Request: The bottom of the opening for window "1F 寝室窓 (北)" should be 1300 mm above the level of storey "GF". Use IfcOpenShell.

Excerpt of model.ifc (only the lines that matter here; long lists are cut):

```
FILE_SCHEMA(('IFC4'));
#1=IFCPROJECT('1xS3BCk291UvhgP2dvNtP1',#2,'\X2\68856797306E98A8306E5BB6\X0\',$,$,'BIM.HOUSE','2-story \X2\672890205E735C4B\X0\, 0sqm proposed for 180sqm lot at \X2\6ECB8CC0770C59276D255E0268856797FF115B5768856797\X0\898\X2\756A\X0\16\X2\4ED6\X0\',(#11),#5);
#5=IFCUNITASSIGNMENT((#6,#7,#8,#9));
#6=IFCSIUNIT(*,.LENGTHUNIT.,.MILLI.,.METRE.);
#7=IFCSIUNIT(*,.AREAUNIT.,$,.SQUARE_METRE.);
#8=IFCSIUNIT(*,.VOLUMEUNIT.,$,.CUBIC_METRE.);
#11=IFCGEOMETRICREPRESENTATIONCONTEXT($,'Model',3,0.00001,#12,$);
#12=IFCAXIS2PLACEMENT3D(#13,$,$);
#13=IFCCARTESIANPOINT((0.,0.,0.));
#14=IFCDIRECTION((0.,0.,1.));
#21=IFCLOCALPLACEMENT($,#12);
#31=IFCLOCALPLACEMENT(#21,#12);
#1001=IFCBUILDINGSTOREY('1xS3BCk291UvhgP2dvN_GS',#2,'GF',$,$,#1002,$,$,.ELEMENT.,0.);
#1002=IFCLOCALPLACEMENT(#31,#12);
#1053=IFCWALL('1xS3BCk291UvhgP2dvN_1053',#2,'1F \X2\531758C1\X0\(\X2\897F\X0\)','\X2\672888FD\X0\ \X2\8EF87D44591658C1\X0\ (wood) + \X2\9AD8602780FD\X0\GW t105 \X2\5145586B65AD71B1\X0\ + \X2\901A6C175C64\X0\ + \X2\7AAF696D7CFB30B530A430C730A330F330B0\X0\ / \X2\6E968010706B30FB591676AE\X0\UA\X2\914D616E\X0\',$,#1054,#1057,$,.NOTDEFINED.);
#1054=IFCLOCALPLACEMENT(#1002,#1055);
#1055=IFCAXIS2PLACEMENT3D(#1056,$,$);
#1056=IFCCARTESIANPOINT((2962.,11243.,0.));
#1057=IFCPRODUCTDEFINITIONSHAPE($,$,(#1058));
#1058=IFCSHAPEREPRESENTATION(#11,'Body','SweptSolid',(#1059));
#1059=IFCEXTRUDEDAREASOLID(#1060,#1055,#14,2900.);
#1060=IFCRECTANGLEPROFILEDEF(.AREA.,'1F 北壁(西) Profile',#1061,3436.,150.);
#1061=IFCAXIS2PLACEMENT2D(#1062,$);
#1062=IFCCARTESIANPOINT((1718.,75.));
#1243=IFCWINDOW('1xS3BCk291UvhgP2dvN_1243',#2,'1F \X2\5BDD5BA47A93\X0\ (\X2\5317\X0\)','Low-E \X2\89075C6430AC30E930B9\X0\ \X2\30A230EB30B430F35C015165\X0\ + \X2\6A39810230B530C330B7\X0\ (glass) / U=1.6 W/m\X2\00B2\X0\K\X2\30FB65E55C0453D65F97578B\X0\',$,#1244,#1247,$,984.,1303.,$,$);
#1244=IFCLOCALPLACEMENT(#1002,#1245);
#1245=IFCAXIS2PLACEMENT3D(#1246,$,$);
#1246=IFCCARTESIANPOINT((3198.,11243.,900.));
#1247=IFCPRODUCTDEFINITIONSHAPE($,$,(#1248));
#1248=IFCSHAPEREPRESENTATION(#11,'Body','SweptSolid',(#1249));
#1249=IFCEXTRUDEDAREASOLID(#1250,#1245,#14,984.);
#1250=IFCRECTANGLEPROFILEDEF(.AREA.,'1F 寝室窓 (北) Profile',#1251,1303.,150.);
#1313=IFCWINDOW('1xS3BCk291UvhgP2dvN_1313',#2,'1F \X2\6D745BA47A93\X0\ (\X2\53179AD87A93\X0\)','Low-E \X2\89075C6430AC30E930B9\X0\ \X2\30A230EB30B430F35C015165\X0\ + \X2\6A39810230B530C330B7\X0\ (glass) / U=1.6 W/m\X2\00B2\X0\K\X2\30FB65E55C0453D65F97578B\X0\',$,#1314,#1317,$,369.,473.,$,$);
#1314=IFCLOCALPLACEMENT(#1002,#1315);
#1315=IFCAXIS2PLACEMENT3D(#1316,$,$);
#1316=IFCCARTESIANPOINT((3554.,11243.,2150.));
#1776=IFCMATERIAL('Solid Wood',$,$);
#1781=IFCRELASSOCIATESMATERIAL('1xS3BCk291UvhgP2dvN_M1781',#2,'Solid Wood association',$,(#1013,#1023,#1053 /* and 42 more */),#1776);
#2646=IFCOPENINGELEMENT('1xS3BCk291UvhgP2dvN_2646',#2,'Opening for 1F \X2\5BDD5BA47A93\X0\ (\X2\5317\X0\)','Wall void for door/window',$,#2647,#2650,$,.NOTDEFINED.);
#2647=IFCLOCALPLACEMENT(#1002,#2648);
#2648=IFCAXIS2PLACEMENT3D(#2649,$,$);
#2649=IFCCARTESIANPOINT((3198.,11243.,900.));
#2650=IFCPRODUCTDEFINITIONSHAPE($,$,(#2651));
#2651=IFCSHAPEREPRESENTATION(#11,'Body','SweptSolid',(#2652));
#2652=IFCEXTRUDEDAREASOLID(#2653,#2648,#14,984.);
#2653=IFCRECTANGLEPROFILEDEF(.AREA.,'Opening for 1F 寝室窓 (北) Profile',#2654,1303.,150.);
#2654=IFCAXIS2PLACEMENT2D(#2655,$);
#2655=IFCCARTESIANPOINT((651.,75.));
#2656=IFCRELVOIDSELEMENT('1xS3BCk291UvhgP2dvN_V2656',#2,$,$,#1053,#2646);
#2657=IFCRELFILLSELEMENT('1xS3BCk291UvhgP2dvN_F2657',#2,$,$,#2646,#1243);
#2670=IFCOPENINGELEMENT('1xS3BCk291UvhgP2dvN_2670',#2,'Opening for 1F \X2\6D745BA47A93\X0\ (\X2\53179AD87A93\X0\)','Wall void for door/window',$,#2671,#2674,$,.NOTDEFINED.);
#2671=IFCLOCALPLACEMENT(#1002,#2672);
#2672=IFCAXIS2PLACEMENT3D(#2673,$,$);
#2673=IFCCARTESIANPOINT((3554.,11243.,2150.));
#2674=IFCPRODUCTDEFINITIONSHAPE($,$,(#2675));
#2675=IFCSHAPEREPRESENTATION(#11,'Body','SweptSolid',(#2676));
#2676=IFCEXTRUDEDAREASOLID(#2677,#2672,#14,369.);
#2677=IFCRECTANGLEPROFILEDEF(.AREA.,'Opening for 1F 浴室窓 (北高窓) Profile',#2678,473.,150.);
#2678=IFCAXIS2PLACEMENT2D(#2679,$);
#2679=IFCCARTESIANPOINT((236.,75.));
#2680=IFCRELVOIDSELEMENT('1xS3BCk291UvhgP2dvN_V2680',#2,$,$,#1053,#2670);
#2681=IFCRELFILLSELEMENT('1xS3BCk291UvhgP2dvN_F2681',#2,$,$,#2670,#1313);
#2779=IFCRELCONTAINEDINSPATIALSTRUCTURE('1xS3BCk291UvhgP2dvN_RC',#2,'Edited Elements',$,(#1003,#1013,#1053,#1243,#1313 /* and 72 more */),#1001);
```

```python
import numpy as np
import ifcopenshell
import ifcopenshell.api.geometry
import ifcopenshell.geom
import ifcopenshell.util.element
import ifcopenshell.util.placement
import ifcopenshell.util.shape
import ifcopenshell.util.unit

model = ifcopenshell.open("model.ifc")
unit_scale = ifcopenshell.util.unit.calculate_unit_scale(model)

window = model.by_guid("1xS3BCk291UvhgP2dvN_1243")
opening = window.FillsVoids[0].RelatingOpeningElement
storey = ifcopenshell.util.element.get_container(window, ifc_class="IfcBuildingStorey")
level = ifcopenshell.util.placement.get_local_placement(storey.ObjectPlacement)[2, 3]

# The opening's origin need not be at the sill, so measure its lowest point.
shape = ifcopenshell.geom.create_shape(ifcopenshell.geom.settings(), opening)
bottom = ifcopenshell.util.shape.get_shape_bottom_elevation(shape, shape.geometry) / unit_scale
dz = level + 1.3 / unit_scale - bottom

shift = np.array([0.0, 0.0, dz])
# The window is not placed relative to its opening, so move both.
for product in (opening, window):
    matrix = ifcopenshell.util.placement.get_local_placement(product.ObjectPlacement)
    matrix[:3, 3] += shift
    ifcopenshell.api.geometry.edit_object_placement(model, product=product, matrix=matrix, is_si=False)

print(f"moved by {dz * unit_scale:+.3f} m")

model.write("model_edited.ifc")
```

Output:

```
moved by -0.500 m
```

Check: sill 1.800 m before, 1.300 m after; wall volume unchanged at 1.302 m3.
